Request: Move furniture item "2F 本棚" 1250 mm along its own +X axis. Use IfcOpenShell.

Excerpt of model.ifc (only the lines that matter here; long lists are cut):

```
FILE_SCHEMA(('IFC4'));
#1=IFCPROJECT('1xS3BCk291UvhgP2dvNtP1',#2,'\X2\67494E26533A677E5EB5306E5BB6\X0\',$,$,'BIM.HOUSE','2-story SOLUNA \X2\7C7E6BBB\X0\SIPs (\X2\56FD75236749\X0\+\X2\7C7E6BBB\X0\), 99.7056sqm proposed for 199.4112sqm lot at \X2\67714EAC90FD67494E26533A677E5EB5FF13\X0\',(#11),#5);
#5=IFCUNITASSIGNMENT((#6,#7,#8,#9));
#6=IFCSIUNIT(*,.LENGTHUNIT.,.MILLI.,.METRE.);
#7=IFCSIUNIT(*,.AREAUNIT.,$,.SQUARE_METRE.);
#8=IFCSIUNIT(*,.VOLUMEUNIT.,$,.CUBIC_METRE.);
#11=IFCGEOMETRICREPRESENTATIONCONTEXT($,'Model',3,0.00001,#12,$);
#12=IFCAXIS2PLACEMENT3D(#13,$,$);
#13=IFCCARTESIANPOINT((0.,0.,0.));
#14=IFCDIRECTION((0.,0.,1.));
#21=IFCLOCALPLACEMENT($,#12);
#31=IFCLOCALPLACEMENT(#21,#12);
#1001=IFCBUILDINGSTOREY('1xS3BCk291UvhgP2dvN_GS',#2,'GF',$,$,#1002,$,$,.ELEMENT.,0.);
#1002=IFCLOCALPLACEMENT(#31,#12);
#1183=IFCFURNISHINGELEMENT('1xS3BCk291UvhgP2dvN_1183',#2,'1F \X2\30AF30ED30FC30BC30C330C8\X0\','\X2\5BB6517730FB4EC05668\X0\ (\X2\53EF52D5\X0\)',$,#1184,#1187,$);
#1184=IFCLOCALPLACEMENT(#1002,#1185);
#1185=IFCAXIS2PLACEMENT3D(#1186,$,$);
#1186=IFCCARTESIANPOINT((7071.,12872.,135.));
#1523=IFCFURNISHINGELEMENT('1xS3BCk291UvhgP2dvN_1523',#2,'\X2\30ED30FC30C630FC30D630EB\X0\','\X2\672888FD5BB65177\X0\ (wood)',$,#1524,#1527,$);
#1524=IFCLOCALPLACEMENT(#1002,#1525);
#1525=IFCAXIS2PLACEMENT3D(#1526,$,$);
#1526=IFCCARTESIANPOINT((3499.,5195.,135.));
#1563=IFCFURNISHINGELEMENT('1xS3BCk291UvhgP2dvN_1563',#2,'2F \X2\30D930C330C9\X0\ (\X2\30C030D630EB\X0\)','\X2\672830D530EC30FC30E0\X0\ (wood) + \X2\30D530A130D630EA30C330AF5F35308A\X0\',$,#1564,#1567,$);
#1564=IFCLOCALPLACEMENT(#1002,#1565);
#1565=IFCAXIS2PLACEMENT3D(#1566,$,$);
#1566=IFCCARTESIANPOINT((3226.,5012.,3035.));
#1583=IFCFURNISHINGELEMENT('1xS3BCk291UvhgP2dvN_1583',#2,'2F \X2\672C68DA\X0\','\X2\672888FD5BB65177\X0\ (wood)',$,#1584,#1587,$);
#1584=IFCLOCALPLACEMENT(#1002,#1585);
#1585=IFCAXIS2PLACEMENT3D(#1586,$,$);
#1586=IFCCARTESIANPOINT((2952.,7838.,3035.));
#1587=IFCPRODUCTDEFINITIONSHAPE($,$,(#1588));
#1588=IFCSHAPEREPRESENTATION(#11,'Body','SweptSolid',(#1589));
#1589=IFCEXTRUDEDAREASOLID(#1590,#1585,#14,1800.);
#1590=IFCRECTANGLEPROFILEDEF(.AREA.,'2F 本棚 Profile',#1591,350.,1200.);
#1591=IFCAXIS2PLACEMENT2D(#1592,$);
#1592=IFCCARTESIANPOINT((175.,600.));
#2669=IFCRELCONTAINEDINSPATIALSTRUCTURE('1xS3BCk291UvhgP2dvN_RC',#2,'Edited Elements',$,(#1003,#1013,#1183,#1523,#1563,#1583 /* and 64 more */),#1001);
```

```python
import ifcopenshell
import ifcopenshell.api.geometry
import ifcopenshell.util.placement
import ifcopenshell.util.unit

model = ifcopenshell.open("model.ifc")
unit_scale = ifcopenshell.util.unit.calculate_unit_scale(model)

item = model.by_guid("1xS3BCk291UvhgP2dvN_1583")
matrix = ifcopenshell.util.placement.get_local_placement(item.ObjectPlacement)
matrix[:3, 3] += matrix[:3, 0] * 1.25 / unit_scale
ifcopenshell.api.geometry.edit_object_placement(model, product=item, matrix=matrix, is_si=False)

print(ifcopenshell.util.placement.get_local_placement(item.ObjectPlacement).round(3) + 0.0)

model.write("model_edited.ifc")
```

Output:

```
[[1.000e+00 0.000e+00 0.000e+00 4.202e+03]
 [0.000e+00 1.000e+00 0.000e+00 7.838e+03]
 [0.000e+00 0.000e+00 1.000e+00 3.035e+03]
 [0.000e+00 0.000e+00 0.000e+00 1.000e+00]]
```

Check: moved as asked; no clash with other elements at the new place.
